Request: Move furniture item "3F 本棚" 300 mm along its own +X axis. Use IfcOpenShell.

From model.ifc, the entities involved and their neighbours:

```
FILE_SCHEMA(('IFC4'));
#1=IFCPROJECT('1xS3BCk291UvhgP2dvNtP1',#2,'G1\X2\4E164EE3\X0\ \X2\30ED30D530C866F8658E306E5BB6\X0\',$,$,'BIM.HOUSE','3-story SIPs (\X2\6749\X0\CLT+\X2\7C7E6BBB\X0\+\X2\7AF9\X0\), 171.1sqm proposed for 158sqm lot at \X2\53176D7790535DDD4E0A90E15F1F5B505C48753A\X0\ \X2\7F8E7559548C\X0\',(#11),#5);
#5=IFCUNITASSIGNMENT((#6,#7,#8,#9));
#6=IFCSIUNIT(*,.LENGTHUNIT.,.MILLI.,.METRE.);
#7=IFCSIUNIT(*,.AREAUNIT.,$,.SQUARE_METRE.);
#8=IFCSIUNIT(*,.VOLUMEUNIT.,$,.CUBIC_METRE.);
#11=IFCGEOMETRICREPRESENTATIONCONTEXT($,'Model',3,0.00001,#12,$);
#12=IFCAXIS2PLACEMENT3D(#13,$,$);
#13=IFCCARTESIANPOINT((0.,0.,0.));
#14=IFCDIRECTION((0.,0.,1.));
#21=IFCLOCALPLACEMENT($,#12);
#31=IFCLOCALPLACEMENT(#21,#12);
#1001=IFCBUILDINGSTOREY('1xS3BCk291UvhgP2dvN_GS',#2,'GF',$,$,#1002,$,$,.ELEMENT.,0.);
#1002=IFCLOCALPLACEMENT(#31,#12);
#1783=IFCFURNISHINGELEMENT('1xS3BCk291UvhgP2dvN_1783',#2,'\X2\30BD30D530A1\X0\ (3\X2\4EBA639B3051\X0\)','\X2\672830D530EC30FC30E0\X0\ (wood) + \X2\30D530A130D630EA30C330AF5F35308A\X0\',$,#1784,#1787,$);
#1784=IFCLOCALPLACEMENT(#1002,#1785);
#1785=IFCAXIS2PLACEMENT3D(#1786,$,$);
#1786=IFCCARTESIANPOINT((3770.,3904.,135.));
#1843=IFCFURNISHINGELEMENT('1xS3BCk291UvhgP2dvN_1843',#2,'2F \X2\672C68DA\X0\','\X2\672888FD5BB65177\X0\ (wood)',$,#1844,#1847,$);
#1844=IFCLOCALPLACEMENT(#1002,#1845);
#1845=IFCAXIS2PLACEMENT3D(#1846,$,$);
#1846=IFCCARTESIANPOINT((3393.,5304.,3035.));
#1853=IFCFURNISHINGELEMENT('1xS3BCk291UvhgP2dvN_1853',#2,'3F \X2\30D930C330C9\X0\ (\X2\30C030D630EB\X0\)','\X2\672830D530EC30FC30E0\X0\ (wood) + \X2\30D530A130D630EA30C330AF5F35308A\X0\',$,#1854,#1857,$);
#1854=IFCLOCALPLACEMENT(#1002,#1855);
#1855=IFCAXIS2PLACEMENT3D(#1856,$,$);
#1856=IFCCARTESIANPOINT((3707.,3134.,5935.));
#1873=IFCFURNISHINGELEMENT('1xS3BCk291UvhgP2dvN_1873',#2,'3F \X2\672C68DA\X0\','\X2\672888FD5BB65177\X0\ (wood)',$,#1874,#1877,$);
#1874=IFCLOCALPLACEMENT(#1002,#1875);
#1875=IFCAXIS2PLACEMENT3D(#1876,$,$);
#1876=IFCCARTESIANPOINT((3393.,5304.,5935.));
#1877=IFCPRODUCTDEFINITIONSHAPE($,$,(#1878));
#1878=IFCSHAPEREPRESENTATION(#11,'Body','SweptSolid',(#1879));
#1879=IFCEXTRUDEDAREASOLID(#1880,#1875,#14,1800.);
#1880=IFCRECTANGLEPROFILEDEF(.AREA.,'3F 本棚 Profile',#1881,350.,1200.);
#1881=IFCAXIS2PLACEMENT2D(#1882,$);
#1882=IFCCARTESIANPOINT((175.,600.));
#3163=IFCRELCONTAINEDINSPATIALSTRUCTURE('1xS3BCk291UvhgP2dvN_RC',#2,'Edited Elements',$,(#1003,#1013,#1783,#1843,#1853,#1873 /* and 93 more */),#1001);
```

```python
import ifcopenshell
import ifcopenshell.api.geometry
import ifcopenshell.util.placement

model = ifcopenshell.open("model.ifc")

item = model.by_guid("1xS3BCk291UvhgP2dvN_1873")
matrix = ifcopenshell.util.placement.get_local_placement(item.ObjectPlacement)
matrix[:3, 3] += matrix[:3, 0] * 300.0
ifcopenshell.api.geometry.edit_object_placement(model, product=item, matrix=matrix, is_si=False)

print(ifcopenshell.util.placement.get_local_placement(item.ObjectPlacement).round(3) + 0.0)

model.write("model_rev.ifc")
```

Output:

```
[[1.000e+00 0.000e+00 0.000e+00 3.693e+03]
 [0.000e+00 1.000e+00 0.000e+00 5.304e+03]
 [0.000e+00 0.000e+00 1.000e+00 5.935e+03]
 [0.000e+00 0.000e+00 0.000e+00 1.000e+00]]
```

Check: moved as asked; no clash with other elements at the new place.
